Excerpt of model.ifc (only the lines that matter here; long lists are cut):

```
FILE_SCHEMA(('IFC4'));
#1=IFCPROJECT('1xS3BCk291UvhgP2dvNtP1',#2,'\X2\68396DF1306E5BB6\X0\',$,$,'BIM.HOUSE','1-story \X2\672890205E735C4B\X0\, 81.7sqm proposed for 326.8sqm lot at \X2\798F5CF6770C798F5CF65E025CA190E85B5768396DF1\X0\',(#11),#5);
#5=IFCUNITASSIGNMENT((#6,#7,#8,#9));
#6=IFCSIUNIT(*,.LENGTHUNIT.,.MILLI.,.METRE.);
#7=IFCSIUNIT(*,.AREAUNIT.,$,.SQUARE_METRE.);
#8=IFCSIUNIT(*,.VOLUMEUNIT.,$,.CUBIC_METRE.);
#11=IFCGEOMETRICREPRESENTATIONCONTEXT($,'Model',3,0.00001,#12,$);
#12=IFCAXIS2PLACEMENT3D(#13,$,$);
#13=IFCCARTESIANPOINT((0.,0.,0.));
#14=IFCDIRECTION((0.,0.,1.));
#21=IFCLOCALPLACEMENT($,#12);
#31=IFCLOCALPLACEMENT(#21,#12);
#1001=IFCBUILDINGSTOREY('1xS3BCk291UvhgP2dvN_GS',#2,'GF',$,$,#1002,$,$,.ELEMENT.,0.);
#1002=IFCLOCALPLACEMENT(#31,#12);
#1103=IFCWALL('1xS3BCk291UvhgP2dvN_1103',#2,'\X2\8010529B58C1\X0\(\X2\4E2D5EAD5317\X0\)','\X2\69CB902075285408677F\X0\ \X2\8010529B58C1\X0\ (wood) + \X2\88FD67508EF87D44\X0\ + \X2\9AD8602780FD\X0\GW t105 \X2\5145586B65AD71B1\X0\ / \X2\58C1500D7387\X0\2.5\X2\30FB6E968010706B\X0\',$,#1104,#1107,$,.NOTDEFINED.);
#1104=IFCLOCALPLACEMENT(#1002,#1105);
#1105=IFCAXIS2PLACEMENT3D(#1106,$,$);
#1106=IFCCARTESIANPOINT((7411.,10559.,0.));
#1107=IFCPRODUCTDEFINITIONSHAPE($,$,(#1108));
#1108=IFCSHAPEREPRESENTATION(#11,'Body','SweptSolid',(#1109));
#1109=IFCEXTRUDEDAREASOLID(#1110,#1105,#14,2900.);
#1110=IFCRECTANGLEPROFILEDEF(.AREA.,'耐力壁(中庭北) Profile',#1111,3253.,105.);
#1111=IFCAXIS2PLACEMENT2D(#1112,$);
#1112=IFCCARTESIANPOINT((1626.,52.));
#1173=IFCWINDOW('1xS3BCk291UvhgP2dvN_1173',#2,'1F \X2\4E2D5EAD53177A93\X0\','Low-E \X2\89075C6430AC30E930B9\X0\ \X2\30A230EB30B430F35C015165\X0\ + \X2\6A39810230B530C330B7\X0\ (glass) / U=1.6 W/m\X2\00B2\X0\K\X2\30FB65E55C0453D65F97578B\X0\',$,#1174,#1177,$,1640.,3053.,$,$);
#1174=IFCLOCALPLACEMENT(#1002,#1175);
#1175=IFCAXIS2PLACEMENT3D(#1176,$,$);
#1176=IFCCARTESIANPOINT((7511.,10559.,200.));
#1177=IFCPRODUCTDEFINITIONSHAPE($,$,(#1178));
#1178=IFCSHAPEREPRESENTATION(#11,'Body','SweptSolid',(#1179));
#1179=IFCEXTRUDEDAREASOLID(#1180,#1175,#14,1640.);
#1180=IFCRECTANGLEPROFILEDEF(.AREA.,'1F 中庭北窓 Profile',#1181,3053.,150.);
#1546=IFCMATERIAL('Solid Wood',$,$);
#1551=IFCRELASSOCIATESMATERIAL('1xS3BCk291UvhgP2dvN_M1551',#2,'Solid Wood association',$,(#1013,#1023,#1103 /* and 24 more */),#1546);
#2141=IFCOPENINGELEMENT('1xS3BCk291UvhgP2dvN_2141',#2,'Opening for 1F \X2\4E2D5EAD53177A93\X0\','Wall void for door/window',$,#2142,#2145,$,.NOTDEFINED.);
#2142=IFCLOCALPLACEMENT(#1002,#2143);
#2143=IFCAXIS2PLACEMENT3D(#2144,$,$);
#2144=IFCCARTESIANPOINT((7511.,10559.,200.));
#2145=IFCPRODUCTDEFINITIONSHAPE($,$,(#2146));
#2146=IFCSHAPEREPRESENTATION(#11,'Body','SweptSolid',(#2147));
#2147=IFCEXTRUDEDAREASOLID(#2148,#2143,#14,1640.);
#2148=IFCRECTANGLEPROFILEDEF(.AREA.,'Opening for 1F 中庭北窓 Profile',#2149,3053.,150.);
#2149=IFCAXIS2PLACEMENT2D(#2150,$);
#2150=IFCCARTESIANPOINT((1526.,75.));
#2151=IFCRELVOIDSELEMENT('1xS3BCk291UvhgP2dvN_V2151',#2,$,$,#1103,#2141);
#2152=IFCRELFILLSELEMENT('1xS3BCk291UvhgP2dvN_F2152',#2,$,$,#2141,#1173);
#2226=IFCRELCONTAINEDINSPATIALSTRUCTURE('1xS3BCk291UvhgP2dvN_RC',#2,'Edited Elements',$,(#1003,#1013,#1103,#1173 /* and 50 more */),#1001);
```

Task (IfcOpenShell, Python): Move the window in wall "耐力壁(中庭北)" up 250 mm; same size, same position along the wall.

```python
import numpy as np
import ifcopenshell
import ifcopenshell.api.geometry
import ifcopenshell.util.placement
import ifcopenshell.util.unit

model = ifcopenshell.open("model.ifc")
unit_scale = ifcopenshell.util.unit.calculate_unit_scale(model)

window = model.by_id(1173)
opening = window.FillsVoids[0].RelatingOpeningElement
dz = 250.0

shift = np.array([0.0, 0.0, dz])
# The window is not placed relative to its opening, so move both.
for product in (opening, window):
    matrix = ifcopenshell.util.placement.get_local_placement(product.ObjectPlacement)
    matrix[:3, 3] += shift
    ifcopenshell.api.geometry.edit_object_placement(model, product=product, matrix=matrix, is_si=False)

print(f"moved by {dz * unit_scale:+.3f} m")

model.write("model_rev.ifc")
```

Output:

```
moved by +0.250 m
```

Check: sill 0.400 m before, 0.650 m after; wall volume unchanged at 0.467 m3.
